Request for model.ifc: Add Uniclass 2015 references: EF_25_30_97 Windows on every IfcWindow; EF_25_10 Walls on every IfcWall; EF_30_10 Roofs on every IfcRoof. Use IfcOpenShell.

First a look at what the model holds.

```python
import ifcopenshell

model = ifcopenshell.open("model.ifc")
print(model.schema)
print("classifications:", [c.Name for c in model.by_type("IfcClassification")])
for ifc_class in ("IfcDoor", "IfcRoof", "IfcStair", "IfcWall", "IfcWindow"):
    print(ifc_class, len(model.by_type(ifc_class)))
```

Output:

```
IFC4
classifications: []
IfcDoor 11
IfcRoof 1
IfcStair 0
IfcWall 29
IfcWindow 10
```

```python
import ifcopenshell
import ifcopenshell.api.classification

model = ifcopenshell.open("model.ifc")

system = ifcopenshell.api.classification.add_classification(model, classification="Uniclass 2015")

codes = {
    "IfcWindow": ("EF_25_30_97", "Windows"),
    "IfcWall": ("EF_25_10", "Walls"),
    "IfcRoof": ("EF_30_10", "Roofs"),
}
for ifc_class, (code, name) in codes.items():
    products = model.by_type(ifc_class)
    ifcopenshell.api.classification.add_reference(
        model, products=products, classification=system, identification=code, name=name
    )
    print(code, len(products))

model.write("model_edited.ifc")
```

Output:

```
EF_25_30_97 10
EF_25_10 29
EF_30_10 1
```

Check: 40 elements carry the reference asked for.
